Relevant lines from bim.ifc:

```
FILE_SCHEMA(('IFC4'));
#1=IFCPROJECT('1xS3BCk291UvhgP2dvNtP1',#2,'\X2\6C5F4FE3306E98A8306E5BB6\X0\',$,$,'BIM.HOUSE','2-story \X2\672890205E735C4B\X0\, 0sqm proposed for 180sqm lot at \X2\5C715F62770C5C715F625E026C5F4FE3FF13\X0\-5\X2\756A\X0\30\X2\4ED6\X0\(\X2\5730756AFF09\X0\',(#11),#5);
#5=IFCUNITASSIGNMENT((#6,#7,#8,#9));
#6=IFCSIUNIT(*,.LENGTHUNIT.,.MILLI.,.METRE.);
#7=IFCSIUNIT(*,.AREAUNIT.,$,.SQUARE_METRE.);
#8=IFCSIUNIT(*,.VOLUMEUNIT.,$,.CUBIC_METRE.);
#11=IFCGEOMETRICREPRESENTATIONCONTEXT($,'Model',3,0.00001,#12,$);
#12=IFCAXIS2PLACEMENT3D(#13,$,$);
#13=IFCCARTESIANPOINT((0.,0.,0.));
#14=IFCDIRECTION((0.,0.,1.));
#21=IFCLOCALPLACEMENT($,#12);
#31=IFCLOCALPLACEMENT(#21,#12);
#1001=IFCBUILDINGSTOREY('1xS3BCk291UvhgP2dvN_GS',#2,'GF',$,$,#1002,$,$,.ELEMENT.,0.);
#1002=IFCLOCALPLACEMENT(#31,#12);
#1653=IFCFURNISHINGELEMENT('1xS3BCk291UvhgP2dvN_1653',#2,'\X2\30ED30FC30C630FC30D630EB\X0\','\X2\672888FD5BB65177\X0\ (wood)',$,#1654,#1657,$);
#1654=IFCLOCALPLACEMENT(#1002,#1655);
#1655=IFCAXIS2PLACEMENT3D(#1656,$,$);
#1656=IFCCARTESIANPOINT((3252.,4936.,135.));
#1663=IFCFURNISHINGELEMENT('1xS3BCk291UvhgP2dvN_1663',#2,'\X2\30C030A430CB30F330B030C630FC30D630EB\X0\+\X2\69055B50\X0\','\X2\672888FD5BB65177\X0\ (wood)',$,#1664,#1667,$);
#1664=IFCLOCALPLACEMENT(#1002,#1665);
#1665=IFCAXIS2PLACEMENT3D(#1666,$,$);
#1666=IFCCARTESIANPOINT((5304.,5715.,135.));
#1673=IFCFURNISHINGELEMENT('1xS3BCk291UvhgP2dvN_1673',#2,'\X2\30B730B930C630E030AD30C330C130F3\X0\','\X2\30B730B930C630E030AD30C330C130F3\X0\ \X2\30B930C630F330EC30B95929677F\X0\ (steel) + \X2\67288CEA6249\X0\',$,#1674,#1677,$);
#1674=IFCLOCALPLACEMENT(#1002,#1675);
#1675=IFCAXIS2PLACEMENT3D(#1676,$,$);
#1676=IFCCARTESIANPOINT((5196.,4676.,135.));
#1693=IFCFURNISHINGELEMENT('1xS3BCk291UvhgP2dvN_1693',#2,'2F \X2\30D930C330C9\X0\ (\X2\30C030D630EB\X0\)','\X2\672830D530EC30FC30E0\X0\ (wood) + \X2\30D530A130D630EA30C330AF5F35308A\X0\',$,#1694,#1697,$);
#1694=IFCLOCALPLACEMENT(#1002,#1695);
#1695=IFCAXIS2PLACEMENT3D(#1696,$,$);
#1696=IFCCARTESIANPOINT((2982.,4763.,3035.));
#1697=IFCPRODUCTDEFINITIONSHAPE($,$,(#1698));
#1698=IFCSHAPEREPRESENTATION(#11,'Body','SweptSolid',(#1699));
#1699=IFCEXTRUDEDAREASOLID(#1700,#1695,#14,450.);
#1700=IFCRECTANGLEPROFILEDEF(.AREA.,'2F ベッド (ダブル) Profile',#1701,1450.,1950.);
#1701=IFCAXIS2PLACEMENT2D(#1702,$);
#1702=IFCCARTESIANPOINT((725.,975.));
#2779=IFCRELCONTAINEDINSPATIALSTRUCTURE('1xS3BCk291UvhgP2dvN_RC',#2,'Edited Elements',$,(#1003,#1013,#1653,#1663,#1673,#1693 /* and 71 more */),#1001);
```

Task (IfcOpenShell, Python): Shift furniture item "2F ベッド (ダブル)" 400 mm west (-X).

```python
import ifcopenshell
import ifcopenshell.api.geometry
import ifcopenshell.util.placement

model = ifcopenshell.open("bim.ifc")

item = model.by_id(1693)
matrix = ifcopenshell.util.placement.get_local_placement(item.ObjectPlacement)
matrix[0, 3] -= 400.0
ifcopenshell.api.geometry.edit_object_placement(model, product=item, matrix=matrix, is_si=False)

print(ifcopenshell.util.placement.get_local_placement(item.ObjectPlacement).round(3) + 0.0)

model.write("bim-out.ifc")
```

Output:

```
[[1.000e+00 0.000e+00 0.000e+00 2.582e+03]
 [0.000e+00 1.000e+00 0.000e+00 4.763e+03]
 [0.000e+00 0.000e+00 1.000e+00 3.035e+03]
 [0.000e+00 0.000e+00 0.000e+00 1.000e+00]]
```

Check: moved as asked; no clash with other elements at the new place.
